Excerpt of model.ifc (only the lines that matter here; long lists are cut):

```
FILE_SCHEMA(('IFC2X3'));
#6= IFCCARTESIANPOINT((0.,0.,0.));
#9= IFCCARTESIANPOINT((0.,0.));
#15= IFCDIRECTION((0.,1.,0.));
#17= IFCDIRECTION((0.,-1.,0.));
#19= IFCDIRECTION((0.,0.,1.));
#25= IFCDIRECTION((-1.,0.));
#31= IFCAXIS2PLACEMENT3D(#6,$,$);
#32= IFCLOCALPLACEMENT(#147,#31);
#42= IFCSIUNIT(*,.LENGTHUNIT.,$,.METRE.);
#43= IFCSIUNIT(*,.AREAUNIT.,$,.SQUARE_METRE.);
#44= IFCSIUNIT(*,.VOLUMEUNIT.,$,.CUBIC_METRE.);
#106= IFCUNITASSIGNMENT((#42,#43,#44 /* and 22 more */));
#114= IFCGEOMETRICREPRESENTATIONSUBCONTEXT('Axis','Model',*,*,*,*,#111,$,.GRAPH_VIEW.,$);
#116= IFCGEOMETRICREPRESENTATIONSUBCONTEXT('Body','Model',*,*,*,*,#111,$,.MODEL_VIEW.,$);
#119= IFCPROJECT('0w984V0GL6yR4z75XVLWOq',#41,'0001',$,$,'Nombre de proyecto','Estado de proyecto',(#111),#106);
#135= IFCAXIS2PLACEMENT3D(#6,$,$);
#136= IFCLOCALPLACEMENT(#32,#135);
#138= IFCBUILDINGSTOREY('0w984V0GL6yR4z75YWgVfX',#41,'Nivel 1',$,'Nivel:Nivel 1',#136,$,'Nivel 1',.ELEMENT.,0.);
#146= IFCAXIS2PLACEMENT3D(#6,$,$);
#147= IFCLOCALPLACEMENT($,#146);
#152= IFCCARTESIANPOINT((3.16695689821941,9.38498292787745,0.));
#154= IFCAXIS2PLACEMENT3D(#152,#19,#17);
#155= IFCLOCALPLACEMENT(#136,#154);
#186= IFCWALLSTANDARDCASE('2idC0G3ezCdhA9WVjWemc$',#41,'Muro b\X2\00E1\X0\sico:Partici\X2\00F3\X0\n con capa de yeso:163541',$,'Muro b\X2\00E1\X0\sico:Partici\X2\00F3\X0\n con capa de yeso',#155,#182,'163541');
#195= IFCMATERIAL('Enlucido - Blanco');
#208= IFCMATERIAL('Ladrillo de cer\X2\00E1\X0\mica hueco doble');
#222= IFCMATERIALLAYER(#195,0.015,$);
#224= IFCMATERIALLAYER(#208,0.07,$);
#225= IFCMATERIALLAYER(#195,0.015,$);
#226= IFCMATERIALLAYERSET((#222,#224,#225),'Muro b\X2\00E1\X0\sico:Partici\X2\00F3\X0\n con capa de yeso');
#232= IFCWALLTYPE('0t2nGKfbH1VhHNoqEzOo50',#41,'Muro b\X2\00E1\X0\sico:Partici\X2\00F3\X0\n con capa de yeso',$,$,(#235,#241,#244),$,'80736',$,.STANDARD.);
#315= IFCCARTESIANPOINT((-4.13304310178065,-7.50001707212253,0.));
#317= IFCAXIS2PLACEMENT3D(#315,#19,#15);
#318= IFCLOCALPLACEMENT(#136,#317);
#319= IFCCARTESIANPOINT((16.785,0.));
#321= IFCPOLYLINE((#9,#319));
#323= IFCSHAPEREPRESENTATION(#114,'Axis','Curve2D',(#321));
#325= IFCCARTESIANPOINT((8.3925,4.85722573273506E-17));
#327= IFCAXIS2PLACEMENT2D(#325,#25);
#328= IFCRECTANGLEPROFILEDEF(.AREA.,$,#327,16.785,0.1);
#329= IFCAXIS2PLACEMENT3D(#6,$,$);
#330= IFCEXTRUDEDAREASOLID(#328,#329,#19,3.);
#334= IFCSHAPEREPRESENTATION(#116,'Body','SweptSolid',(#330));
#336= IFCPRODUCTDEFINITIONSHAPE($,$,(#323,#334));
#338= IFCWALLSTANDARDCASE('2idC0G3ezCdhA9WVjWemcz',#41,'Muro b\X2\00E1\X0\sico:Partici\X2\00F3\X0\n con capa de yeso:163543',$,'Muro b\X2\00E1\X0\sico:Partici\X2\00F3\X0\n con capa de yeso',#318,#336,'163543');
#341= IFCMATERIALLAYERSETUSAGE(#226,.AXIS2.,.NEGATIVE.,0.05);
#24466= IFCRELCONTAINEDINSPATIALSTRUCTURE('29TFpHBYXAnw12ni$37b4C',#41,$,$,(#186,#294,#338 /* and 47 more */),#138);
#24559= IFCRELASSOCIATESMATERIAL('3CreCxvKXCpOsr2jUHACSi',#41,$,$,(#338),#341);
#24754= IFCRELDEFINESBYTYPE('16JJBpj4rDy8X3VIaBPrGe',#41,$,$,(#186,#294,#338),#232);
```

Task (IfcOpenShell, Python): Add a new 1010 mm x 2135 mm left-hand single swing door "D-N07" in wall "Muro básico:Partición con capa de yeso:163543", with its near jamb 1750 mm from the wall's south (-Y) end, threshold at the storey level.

```python
import numpy as np
import ifcopenshell
import ifcopenshell.api.feature
import ifcopenshell.api.geometry
import ifcopenshell.api.root
import ifcopenshell.api.spatial
import ifcopenshell.api.type
import ifcopenshell.geom
import ifcopenshell.util.element
import ifcopenshell.util.placement
import ifcopenshell.util.representation
import ifcopenshell.util.shape
import ifcopenshell.util.unit

model = ifcopenshell.open("model.ifc")
unit_scale = ifcopenshell.util.unit.calculate_unit_scale(model)
settings = ifcopenshell.geom.settings()


def volume(element):
    """Net volume in cubic metres, openings subtracted."""
    shape = ifcopenshell.geom.create_shape(settings, element)
    return ifcopenshell.util.shape.get_volume(shape.geometry)


wall = model.by_guid("2idC0G3ezCdhA9WVjWemcz")
storey = ifcopenshell.util.element.get_container(wall, ifc_class="IfcBuildingStorey")
context = ifcopenshell.util.representation.get_context(model, "Model", "Body", "MODEL_VIEW")
before = volume(wall)

width, height, from_end, sill = 1.01, 2.135, 1.75, 0.0  # metres

# The wall runs along its own X axis, and the end named is its -X end.
wall_shape = ifcopenshell.geom.create_shape(settings, wall)
x, y, z = ifcopenshell.util.shape.get_vertices(wall_shape.geometry).T
start = x.min() + from_end
face, thickness = float(y.min()), float(y.max() - y.min())
wall_matrix = ifcopenshell.util.placement.get_local_placement(wall.ObjectPlacement)
level = ifcopenshell.util.placement.get_local_placement(storey.ObjectPlacement)[2, 3]


def in_wall(x, y):
    """Placement at x, y metres in the wall's axes, at sill height."""
    matrix = wall_matrix.copy()
    matrix[:, 3] = wall_matrix @ np.array([x / unit_scale, y / unit_scale, 0.0, 1.0])
    matrix[2, 3] = level + sill / unit_scale
    return matrix


# Opening: a box that overshoots both wall faces by 50 mm.
opening = ifcopenshell.api.root.create_entity(model, ifc_class="IfcOpeningElement")
box = ifcopenshell.api.geometry.add_wall_representation(
    model, context=context, length=width, height=height, thickness=thickness + 0.1
)
ifcopenshell.api.geometry.assign_representation(model, product=opening, representation=box)
ifcopenshell.api.geometry.edit_object_placement(model, product=opening, matrix=in_wall(start, face - 0.05), is_si=False)
ifcopenshell.api.feature.add_feature(model, feature=opening, element=wall)

door = ifcopenshell.api.root.create_entity(model, ifc_class="IfcDoor", name="D-N07")
door.OverallWidth, door.OverallHeight = width / unit_scale, height / unit_scale
body = ifcopenshell.api.geometry.add_door_representation(
    model,
    context=context,
    overall_width=door.OverallWidth,
    overall_height=door.OverallHeight,
    operation_type="SINGLE_SWING_LEFT",
    lining_properties={"LiningDepth": thickness / unit_scale, "ThresholdDepth": thickness / unit_scale},
)
ifcopenshell.api.geometry.assign_representation(model, product=door, representation=body)
ifcopenshell.api.spatial.assign_container(model, products=[door], relating_structure=storey)
fills = ifcopenshell.api.feature.add_filling(model, opening=opening, element=door)
fills.OwnerHistory = door.OwnerHistory  # required in IFC2X3

# IFC2X3 keeps the operation on the door style.
style = ifcopenshell.api.root.create_entity(model, ifc_class="IfcDoorStyle", name="D-N07")
style.OperationType, style.ConstructionType = "SINGLE_SWING_LEFT", "NOTDEFINED"
style.ParameterTakesPrecedence = style.Sizeable = False
ifcopenshell.api.type.assign_type(model, related_objects=[door], relating_type=style)

# The lining spans the wall, so the door starts at the wall face.
ifcopenshell.api.geometry.edit_object_placement(model, product=door, matrix=in_wall(start, face), is_si=False)

after = volume(wall)

print(f"wall volume {before:.3f} -> {after:.3f} m3")

model.write("model_rev.ifc")
```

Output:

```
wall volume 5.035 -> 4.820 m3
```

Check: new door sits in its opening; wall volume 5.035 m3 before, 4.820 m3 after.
